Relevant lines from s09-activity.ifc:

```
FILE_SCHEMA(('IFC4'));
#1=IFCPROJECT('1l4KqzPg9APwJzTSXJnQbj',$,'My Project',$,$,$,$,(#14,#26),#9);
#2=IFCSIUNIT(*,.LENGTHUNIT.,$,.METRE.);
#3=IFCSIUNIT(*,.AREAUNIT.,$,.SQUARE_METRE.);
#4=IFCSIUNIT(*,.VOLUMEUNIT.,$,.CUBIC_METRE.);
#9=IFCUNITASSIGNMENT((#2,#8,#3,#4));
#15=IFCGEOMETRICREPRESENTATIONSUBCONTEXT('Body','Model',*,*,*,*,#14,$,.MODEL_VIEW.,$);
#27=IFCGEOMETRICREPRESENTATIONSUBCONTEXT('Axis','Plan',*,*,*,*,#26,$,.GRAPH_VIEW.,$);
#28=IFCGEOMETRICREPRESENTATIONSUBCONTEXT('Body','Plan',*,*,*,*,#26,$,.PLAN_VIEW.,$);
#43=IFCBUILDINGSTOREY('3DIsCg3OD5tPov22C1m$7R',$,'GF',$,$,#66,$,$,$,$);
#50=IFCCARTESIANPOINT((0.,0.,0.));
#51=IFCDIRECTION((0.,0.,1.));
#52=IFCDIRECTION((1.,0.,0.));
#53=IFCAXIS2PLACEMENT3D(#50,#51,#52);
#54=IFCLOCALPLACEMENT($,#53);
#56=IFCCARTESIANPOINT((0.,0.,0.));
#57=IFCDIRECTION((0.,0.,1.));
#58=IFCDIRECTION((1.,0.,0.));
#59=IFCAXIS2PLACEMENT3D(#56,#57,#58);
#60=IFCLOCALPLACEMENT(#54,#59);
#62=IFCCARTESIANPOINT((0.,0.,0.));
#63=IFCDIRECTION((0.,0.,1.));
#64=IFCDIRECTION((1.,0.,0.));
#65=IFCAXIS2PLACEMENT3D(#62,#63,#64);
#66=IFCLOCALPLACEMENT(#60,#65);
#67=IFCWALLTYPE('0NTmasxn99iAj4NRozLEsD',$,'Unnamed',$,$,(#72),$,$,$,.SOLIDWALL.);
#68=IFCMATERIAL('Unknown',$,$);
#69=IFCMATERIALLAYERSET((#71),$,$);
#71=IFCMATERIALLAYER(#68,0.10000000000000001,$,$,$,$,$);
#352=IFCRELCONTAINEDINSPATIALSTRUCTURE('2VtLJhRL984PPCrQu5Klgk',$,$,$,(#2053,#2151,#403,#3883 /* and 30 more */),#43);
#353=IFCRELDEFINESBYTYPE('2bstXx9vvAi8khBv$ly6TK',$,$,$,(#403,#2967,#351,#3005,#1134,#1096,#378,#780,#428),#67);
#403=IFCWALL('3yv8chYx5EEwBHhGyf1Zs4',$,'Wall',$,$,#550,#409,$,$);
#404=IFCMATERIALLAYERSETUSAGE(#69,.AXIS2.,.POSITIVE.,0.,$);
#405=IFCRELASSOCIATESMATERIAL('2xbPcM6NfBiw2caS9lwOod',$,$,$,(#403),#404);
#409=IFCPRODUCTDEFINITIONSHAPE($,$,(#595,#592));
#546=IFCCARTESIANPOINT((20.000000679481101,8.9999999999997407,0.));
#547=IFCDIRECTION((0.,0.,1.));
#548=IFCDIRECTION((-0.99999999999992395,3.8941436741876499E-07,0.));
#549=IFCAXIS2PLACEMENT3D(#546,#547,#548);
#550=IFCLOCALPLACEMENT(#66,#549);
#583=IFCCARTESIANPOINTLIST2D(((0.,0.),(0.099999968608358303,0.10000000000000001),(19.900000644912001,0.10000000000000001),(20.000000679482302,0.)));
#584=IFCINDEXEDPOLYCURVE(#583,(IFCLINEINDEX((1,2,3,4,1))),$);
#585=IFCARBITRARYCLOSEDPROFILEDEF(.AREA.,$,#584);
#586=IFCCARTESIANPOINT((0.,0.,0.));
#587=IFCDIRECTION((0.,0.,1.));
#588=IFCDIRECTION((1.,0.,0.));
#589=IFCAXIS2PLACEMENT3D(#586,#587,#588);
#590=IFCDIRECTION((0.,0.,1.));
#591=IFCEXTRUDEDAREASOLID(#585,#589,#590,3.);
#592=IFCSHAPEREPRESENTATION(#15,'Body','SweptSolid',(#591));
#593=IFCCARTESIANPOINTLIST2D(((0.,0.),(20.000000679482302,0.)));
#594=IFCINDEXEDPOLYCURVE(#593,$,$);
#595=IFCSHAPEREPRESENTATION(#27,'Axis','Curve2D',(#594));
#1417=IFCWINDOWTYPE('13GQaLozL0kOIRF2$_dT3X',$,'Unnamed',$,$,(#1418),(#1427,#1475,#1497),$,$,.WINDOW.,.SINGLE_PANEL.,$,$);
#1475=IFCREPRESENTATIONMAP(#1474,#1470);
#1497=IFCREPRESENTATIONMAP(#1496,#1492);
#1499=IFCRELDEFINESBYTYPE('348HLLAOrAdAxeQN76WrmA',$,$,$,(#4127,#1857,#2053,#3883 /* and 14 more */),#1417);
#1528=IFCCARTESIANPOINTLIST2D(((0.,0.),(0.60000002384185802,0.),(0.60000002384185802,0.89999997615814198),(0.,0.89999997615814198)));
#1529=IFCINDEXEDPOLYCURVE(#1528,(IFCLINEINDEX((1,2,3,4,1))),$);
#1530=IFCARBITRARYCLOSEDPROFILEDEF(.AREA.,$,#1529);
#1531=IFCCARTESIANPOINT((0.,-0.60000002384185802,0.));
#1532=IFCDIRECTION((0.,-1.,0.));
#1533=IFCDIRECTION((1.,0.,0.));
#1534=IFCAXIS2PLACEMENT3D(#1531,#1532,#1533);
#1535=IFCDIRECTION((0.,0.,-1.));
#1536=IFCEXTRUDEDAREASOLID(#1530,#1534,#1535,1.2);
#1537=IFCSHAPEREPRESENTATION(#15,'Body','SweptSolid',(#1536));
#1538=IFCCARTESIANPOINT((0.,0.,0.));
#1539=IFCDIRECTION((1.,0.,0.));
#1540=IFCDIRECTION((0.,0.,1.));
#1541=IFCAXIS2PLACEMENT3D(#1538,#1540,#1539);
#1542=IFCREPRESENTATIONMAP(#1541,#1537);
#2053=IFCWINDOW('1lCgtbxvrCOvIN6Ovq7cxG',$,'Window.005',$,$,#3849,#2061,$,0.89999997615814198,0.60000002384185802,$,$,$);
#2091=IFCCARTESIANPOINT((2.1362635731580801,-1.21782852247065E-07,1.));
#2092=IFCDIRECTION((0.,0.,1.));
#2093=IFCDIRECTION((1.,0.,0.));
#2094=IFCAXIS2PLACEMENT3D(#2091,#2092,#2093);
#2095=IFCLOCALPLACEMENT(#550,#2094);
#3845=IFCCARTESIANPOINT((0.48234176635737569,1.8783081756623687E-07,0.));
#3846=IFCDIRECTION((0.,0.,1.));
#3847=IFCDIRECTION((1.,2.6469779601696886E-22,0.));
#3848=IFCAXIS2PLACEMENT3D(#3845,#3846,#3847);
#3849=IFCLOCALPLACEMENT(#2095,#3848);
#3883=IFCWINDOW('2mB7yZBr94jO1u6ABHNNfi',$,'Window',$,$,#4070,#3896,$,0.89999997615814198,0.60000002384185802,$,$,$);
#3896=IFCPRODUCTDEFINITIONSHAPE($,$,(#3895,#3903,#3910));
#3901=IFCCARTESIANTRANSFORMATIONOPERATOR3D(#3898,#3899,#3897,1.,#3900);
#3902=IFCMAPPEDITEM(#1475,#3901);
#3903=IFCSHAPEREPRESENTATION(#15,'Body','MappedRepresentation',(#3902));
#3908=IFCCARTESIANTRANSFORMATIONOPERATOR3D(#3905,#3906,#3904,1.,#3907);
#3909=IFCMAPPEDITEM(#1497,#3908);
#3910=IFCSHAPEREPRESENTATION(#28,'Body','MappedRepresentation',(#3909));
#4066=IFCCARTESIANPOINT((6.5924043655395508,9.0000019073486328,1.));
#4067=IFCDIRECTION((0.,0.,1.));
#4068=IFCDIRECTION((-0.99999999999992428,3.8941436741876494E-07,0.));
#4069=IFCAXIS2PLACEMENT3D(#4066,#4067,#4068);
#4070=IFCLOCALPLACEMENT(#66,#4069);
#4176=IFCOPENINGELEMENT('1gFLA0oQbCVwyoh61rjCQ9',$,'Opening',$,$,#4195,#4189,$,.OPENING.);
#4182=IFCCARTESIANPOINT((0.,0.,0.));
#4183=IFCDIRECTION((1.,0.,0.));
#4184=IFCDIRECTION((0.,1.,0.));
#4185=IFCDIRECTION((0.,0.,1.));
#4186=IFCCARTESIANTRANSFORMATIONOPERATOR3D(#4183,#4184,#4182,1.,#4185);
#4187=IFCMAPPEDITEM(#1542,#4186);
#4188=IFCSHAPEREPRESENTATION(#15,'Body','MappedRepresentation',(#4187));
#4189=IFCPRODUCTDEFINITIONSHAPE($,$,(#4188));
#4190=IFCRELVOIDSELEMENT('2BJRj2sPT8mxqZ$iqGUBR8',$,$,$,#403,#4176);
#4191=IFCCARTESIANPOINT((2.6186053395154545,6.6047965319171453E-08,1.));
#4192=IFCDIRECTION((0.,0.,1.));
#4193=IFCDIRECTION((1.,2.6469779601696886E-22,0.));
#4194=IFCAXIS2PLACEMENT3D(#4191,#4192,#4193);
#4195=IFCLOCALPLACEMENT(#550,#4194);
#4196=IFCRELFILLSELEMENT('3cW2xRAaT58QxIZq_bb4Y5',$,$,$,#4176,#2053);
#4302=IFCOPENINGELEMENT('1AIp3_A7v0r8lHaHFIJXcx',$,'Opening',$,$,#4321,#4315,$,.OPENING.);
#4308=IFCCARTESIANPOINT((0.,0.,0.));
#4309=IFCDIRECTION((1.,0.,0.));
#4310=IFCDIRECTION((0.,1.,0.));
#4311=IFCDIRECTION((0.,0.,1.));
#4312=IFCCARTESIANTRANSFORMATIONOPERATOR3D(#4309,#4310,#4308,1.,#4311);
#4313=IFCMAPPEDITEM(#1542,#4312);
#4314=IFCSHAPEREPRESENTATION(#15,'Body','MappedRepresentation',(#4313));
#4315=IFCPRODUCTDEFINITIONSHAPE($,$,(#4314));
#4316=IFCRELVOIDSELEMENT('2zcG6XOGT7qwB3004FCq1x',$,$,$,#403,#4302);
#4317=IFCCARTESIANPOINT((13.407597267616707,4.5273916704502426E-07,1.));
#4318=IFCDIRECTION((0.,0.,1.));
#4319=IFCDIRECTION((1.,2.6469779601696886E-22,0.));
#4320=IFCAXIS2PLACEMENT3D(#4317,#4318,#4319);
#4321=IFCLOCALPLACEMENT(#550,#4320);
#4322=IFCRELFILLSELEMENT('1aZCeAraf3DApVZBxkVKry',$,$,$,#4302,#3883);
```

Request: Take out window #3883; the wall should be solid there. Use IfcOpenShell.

```python
import ifcopenshell
import ifcopenshell.api.feature
import ifcopenshell.api.root
import ifcopenshell.geom
import ifcopenshell.util.shape

model = ifcopenshell.open("s09-activity.ifc")
settings = ifcopenshell.geom.settings()


def volume(element):
    """Net volume in cubic metres, openings subtracted."""
    shape = ifcopenshell.geom.create_shape(settings, element)
    return ifcopenshell.util.shape.get_volume(shape.geometry)


window = model.by_guid("2mB7yZBr94jO1u6ABHNNfi")
opening = window.FillsVoids[0].RelatingOpeningElement
wall = opening.VoidsElements[0].RelatingBuildingElement
before = volume(wall)

ifcopenshell.api.root.remove_product(model, product=window)
ifcopenshell.api.feature.remove_feature(model, feature=opening)

after = volume(wall)

print(f"wall volume {before:.3f} -> {after:.3f} m3")

model.write("s09-activity_v2.ifc")
```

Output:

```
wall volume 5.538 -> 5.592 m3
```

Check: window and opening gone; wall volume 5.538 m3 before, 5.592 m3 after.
